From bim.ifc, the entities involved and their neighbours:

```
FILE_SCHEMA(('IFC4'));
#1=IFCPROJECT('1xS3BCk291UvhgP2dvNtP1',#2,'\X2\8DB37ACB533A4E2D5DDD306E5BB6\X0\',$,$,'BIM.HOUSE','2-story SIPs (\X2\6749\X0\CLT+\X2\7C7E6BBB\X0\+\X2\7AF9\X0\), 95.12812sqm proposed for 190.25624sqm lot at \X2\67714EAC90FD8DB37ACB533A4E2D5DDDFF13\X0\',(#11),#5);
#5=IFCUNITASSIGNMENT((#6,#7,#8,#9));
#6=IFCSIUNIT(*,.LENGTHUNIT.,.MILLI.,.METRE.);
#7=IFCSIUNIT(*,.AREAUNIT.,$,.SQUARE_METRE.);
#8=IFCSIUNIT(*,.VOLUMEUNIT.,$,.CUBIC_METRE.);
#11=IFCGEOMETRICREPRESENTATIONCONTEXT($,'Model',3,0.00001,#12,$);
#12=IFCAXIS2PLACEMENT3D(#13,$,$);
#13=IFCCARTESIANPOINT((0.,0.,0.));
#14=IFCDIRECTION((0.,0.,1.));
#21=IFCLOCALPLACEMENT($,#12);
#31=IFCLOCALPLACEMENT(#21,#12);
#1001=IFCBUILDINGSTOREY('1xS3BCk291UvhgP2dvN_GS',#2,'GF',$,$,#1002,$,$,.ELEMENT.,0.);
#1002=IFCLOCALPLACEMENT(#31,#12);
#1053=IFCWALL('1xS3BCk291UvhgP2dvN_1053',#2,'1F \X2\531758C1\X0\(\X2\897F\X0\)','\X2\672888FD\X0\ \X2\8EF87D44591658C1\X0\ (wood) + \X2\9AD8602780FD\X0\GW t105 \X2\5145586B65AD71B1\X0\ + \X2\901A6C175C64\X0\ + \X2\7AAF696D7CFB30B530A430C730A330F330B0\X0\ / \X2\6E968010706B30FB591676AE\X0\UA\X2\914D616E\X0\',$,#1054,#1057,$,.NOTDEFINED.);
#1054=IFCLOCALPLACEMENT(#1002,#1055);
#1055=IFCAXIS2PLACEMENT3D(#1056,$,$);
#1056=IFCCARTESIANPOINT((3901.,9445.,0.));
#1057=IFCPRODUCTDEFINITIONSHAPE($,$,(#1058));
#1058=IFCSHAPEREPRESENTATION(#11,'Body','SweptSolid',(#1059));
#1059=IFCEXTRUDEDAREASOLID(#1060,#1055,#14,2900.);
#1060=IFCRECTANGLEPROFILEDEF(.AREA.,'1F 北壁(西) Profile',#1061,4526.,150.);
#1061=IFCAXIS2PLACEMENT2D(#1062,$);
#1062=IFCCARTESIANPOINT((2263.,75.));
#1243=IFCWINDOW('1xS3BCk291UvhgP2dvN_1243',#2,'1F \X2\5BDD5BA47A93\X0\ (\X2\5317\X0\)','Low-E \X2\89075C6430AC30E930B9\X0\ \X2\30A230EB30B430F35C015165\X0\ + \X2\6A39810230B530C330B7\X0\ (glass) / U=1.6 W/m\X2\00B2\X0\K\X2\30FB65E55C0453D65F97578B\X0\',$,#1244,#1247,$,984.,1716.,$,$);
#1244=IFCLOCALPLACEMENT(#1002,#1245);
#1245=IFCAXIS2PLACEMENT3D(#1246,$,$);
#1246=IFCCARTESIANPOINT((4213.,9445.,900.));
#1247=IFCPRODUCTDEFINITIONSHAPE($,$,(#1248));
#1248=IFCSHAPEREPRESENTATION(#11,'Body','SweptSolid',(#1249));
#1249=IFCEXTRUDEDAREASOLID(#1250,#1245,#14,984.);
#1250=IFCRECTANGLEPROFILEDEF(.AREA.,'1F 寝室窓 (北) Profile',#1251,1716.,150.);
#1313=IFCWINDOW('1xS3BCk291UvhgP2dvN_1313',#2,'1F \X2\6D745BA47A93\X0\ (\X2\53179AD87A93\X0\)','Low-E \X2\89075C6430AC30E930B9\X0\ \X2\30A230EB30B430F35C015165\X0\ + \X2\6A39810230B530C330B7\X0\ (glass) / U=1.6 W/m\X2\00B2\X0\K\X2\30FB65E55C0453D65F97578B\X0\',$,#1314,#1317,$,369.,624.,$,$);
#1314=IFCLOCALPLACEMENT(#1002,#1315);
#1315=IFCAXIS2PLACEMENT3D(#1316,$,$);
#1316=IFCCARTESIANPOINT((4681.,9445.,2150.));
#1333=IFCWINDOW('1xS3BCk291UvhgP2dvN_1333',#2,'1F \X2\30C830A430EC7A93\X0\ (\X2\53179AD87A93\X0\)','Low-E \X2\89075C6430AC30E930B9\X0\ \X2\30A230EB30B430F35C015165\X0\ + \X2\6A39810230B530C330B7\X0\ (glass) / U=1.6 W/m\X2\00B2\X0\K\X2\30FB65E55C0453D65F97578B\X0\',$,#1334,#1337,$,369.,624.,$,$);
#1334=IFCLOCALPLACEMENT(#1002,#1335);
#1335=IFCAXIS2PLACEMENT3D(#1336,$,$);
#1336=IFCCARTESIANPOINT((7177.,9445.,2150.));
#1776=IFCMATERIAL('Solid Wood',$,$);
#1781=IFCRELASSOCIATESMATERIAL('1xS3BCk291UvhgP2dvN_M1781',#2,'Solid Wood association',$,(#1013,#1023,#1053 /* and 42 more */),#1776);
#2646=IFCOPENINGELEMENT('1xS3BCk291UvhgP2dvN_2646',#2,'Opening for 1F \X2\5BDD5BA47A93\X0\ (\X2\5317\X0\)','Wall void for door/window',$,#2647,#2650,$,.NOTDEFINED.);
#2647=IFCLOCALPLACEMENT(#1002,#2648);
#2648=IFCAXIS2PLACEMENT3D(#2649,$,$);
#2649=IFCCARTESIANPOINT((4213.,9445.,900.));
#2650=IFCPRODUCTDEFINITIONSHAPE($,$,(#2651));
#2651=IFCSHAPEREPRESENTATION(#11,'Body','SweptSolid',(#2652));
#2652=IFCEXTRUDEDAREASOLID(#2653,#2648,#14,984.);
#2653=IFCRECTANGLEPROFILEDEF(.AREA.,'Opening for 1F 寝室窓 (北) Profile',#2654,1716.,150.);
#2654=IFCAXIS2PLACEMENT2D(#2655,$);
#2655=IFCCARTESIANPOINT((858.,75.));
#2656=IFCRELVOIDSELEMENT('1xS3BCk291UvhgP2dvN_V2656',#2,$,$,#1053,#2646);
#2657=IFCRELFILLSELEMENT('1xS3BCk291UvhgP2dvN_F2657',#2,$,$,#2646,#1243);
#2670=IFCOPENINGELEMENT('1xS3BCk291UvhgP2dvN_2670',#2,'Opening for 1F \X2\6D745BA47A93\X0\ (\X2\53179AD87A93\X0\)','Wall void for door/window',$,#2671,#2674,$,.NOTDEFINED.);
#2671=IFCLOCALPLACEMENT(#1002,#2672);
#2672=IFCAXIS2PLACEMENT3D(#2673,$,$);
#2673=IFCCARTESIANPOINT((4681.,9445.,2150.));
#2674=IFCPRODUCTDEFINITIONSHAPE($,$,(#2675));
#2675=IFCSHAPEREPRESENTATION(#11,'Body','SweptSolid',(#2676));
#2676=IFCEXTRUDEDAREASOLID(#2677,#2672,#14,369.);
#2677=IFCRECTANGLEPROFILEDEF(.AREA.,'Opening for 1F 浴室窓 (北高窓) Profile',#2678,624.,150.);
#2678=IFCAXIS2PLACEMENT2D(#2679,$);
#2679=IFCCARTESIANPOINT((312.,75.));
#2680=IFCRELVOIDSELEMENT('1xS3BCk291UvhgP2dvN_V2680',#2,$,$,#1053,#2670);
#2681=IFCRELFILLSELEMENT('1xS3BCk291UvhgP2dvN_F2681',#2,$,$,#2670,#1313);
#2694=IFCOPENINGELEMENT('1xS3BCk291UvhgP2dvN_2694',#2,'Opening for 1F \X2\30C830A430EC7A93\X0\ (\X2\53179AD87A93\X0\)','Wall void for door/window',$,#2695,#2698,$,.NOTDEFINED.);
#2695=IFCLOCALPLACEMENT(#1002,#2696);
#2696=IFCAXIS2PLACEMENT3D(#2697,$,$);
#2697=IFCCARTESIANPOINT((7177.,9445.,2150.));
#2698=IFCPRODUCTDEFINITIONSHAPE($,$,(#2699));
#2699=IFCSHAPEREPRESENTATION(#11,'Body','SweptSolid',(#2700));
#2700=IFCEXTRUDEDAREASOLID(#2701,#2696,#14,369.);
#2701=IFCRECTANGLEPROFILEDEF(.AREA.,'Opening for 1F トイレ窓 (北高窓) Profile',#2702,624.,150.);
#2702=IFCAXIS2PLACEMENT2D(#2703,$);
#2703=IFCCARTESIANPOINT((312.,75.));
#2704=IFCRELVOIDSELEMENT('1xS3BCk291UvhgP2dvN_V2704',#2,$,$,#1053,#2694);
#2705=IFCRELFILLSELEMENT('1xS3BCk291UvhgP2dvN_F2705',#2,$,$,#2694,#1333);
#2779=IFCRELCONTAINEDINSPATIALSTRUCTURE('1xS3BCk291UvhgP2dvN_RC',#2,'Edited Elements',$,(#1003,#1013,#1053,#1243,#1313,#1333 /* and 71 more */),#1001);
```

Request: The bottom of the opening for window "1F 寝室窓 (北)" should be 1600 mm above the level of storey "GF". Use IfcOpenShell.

```python
import numpy as np
import ifcopenshell
import ifcopenshell.api.geometry
import ifcopenshell.geom
import ifcopenshell.util.element
import ifcopenshell.util.placement
import ifcopenshell.util.shape
import ifcopenshell.util.unit

model = ifcopenshell.open("bim.ifc")
unit_scale = ifcopenshell.util.unit.calculate_unit_scale(model)

window = model.by_guid("1xS3BCk291UvhgP2dvN_1243")
opening = window.FillsVoids[0].RelatingOpeningElement
storey = ifcopenshell.util.element.get_container(window, ifc_class="IfcBuildingStorey")
level = ifcopenshell.util.placement.get_local_placement(storey.ObjectPlacement)[2, 3]

# The opening's origin need not be at the sill, so measure its lowest point.
shape = ifcopenshell.geom.create_shape(ifcopenshell.geom.settings(), opening)
bottom = ifcopenshell.util.shape.get_shape_bottom_elevation(shape, shape.geometry) / unit_scale
dz = level + 1.6 / unit_scale - bottom

shift = np.array([0.0, 0.0, dz])
# The window is not placed relative to its opening, so move both.
for product in (opening, window):
    matrix = ifcopenshell.util.placement.get_local_placement(product.ObjectPlacement)
    matrix[:3, 3] += shift
    ifcopenshell.api.geometry.edit_object_placement(model, product=product, matrix=matrix, is_si=False)

print(f"moved by {dz * unit_scale:+.3f} m")

model.write("bim_v2.ifc")
```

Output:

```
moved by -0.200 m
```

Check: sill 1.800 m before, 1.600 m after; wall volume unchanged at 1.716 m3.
